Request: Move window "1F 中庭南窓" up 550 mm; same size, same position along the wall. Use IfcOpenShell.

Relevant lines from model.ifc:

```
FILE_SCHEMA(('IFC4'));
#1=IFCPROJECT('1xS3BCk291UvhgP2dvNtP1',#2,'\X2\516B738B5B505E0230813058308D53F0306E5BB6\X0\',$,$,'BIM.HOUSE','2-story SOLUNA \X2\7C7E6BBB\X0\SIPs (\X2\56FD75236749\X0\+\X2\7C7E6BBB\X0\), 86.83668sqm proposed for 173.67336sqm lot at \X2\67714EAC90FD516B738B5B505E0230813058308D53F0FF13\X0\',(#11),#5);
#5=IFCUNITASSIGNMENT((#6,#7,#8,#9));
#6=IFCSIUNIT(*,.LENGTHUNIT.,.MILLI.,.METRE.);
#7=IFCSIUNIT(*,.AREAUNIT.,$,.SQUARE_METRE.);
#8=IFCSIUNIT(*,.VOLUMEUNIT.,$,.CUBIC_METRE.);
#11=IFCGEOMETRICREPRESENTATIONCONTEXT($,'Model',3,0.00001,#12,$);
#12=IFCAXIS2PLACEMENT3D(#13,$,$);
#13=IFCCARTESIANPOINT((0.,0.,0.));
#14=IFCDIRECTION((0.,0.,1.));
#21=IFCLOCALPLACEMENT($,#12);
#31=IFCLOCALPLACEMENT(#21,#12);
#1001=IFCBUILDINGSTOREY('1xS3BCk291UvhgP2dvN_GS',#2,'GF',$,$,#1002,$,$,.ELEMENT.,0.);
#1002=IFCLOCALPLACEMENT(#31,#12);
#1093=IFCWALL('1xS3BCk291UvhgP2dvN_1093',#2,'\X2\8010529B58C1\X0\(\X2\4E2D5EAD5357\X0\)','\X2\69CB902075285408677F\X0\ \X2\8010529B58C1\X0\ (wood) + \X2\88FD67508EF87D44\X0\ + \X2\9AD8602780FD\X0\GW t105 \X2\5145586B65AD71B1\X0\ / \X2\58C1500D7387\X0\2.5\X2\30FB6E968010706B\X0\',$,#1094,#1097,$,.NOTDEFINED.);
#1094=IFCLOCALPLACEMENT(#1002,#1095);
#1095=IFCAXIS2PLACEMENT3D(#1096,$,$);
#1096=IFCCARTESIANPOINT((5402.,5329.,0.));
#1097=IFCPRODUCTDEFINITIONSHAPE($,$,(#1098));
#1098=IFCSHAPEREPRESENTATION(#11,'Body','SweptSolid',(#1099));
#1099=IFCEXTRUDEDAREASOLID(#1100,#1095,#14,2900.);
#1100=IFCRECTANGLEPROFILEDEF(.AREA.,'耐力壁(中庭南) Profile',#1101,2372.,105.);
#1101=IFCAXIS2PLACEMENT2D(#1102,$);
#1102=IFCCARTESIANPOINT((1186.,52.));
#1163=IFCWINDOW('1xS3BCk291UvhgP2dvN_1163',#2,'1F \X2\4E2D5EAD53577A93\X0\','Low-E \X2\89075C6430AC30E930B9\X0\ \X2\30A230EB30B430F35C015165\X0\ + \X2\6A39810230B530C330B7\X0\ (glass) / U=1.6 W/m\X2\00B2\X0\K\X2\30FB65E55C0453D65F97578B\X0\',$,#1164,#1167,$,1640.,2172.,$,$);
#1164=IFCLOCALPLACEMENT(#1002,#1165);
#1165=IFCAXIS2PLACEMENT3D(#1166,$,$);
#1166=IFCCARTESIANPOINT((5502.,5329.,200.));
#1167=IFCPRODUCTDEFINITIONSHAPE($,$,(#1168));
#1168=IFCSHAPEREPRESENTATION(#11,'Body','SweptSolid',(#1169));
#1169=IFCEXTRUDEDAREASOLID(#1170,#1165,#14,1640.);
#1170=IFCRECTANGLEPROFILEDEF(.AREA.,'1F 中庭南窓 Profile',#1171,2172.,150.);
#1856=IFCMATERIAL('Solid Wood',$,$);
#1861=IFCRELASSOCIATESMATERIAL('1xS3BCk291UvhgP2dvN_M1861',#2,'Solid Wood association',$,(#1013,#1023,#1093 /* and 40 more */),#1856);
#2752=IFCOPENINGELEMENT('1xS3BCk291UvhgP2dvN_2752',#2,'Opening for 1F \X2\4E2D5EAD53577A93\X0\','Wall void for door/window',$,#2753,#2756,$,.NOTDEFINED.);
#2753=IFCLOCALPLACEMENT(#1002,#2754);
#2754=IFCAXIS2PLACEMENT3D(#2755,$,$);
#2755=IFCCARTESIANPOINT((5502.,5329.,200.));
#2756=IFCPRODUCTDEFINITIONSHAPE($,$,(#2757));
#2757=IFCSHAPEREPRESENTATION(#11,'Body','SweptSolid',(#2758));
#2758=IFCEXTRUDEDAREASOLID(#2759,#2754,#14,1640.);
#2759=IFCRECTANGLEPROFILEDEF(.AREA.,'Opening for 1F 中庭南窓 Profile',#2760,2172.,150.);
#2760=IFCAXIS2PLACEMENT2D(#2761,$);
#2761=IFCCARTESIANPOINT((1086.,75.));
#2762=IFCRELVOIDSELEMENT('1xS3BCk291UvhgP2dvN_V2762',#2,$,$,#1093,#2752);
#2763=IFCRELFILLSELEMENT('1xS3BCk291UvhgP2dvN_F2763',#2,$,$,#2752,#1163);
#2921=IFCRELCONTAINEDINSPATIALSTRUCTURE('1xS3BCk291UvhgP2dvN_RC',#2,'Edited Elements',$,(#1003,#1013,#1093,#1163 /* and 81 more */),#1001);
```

```python
import numpy as np
import ifcopenshell
import ifcopenshell.api.geometry
import ifcopenshell.util.placement
import ifcopenshell.util.unit

model = ifcopenshell.open("model.ifc")
unit_scale = ifcopenshell.util.unit.calculate_unit_scale(model)

window = model.by_id(1163)
opening = window.FillsVoids[0].RelatingOpeningElement
dz = 550.0

shift = np.array([0.0, 0.0, dz])
# The window is not placed relative to its opening, so move both.
for product in (opening, window):
    matrix = ifcopenshell.util.placement.get_local_placement(product.ObjectPlacement)
    matrix[:3, 3] += shift
    ifcopenshell.api.geometry.edit_object_placement(model, product=product, matrix=matrix, is_si=False)

print(f"moved by {dz * unit_scale:+.3f} m")

model.write("model_updated.ifc")
```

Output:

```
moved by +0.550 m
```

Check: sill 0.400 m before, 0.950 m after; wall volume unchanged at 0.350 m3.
